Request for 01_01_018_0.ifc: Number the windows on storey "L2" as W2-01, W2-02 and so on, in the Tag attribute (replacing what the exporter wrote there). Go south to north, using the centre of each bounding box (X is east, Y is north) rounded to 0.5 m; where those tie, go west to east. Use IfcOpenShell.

First a look at what the model holds.

```python
import ifcopenshell
import ifcopenshell.util.element
import ifcopenshell.util.placement

model = ifcopenshell.open("01_01_018_0.ifc")
print(model.schema)
storey = next(s for s in model.by_type("IfcBuildingStorey") if s.Name == "L2")
windows = [e for e in ifcopenshell.util.element.get_decomposition(storey) if e.is_a("IfcWindow")]
for e in sorted(windows, key=lambda e: e.id()):
    origin = ifcopenshell.util.placement.get_local_placement(e.ObjectPlacement)[:3, 3]
    print(e.id(), e.Tag, e.Name, origin.round(2) + 0.0, sep=" | ")
```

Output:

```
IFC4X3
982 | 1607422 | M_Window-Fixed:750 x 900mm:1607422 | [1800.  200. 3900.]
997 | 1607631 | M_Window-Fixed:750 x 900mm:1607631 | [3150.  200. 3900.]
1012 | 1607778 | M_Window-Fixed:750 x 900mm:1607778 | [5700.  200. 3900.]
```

```python
import ifcopenshell
import ifcopenshell.geom
import ifcopenshell.util.element
import ifcopenshell.util.shape

model = ifcopenshell.open("01_01_018_0.ifc")
settings = ifcopenshell.geom.settings()
settings.set("use-world-coords", True)


def centre(element):
    shape = ifcopenshell.geom.create_shape(settings, element)
    return ifcopenshell.util.shape.get_bbox_centroid(shape.geometry)


storey = next(s for s in model.by_type("IfcBuildingStorey") if s.Name == "L2")
windows = [e for e in ifcopenshell.util.element.get_decomposition(storey) if e.is_a("IfcWindow")]

# Insertion points can sit at a corner or the storey origin, so sort by the geometry (in metres).
centres = {e: centre(e) for e in windows}
windows.sort(key=lambda e: (round(centres[e][1] / 0.5), centres[e][0]))

for i, e in enumerate(windows, start=1):
    number = f"W2-{i:02d}"
    e.Tag = number
    print(e.id(), number)

model.write("01_01_018_0_updated.ifc")
```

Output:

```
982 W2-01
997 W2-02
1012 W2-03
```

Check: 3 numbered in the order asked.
